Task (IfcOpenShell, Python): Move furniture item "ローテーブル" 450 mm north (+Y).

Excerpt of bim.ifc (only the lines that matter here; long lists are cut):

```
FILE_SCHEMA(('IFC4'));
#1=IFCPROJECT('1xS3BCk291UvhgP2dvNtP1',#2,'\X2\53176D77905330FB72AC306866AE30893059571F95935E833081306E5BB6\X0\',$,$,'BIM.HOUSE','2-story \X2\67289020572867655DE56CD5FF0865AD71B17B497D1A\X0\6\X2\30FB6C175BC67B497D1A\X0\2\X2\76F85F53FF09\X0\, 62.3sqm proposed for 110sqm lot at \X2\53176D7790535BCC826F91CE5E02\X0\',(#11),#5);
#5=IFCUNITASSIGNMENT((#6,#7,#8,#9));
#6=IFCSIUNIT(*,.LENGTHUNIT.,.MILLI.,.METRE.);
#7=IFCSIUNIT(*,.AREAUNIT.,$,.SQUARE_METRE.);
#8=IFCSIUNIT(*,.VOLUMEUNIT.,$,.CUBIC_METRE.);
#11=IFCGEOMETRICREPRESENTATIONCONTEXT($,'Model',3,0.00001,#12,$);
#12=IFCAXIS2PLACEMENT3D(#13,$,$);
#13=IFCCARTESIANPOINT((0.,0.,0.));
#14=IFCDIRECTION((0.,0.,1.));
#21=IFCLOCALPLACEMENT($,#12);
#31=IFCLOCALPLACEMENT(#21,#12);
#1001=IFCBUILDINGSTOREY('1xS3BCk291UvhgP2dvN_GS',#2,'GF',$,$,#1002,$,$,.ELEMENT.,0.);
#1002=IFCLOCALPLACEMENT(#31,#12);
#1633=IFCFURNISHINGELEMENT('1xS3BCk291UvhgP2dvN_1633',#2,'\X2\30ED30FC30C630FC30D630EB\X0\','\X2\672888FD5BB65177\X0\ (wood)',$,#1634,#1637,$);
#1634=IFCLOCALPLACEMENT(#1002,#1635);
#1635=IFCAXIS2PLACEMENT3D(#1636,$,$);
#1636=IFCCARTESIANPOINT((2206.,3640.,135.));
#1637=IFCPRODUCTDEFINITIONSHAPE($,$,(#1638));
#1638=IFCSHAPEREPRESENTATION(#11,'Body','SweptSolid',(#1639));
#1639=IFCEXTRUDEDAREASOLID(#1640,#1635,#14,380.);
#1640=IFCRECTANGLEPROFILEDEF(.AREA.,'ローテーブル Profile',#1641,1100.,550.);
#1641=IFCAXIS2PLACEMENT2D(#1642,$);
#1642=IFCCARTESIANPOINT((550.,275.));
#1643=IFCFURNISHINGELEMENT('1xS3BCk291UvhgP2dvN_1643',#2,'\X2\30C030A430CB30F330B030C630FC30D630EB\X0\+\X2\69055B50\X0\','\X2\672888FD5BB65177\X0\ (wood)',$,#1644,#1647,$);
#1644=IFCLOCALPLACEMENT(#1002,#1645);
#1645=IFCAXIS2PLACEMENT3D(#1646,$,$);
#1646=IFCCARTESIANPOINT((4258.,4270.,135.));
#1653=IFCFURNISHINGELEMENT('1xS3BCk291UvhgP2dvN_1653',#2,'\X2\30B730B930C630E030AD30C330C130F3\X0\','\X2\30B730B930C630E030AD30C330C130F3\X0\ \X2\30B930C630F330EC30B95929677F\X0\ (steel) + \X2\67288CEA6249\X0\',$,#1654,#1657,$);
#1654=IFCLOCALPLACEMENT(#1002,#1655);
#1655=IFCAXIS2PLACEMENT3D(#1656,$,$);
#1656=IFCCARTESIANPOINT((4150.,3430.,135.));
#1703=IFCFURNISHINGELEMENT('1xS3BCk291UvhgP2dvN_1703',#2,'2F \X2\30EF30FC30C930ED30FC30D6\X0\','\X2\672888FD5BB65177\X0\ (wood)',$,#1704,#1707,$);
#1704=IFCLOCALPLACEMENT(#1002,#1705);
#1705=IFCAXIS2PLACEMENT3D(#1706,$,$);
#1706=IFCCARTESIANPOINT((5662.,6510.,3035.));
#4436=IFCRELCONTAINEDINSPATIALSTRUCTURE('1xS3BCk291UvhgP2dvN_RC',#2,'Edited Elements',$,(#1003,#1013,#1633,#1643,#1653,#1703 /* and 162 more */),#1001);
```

```python
import ifcopenshell
import ifcopenshell.api.geometry
import ifcopenshell.util.placement
import ifcopenshell.util.unit

model = ifcopenshell.open("bim.ifc")
unit_scale = ifcopenshell.util.unit.calculate_unit_scale(model)

item = model.by_guid("1xS3BCk291UvhgP2dvN_1633")
matrix = ifcopenshell.util.placement.get_local_placement(item.ObjectPlacement)
matrix[1, 3] += 0.45 / unit_scale
ifcopenshell.api.geometry.edit_object_placement(model, product=item, matrix=matrix, is_si=False)

print(ifcopenshell.util.placement.get_local_placement(item.ObjectPlacement).round(3) + 0.0)

model.write("bim_updated.ifc")
```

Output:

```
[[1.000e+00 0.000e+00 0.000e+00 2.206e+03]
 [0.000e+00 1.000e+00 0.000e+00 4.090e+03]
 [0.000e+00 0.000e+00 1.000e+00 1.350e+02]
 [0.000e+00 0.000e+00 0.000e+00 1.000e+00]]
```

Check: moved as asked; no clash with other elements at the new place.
